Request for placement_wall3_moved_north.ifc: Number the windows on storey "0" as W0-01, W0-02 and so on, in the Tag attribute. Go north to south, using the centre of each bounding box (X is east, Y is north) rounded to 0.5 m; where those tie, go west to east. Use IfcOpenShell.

First a look at what the model holds.

```python
import ifcopenshell
import ifcopenshell.util.element
import ifcopenshell.util.placement

model = ifcopenshell.open("placement_wall3_moved_north.ifc")
print(model.schema)
storey = next(s for s in model.by_type("IfcBuildingStorey") if s.Name == "0")
windows = [e for e in ifcopenshell.util.element.get_decomposition(storey) if e.is_a("IfcWindow")]
for e in sorted(windows, key=lambda e: e.id()):
    origin = ifcopenshell.util.placement.get_local_placement(e.ObjectPlacement)[:3, 3]
    print(e.id(), e.Tag, e.Name, origin.round(2) + 0.0, sep=" | ")
```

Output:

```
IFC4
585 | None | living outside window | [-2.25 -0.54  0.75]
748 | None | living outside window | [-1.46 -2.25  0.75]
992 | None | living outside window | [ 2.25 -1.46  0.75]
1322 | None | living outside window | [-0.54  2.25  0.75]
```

```python
import ifcopenshell
import ifcopenshell.geom
import ifcopenshell.util.element
import ifcopenshell.util.shape

model = ifcopenshell.open("placement_wall3_moved_north.ifc")
settings = ifcopenshell.geom.settings()
settings.set("use-world-coords", True)


def centre(element):
    shape = ifcopenshell.geom.create_shape(settings, element)
    return ifcopenshell.util.shape.get_bbox_centroid(shape.geometry)


storey = next(s for s in model.by_type("IfcBuildingStorey") if s.Name == "0")
windows = [e for e in ifcopenshell.util.element.get_decomposition(storey) if e.is_a("IfcWindow")]

# Insertion points can sit at a corner or the storey origin, so sort by the geometry (in metres).
centres = {e: centre(e) for e in windows}
windows.sort(key=lambda e: (-round(centres[e][1] / 0.5), centres[e][0]))

for i, e in enumerate(windows, start=1):
    number = f"W0-{i:02d}"
    e.Tag = number
    print(e.id(), number)

model.write("placement_wall3_moved_north_rev.ifc")
```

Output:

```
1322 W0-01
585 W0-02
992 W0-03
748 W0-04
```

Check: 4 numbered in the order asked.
